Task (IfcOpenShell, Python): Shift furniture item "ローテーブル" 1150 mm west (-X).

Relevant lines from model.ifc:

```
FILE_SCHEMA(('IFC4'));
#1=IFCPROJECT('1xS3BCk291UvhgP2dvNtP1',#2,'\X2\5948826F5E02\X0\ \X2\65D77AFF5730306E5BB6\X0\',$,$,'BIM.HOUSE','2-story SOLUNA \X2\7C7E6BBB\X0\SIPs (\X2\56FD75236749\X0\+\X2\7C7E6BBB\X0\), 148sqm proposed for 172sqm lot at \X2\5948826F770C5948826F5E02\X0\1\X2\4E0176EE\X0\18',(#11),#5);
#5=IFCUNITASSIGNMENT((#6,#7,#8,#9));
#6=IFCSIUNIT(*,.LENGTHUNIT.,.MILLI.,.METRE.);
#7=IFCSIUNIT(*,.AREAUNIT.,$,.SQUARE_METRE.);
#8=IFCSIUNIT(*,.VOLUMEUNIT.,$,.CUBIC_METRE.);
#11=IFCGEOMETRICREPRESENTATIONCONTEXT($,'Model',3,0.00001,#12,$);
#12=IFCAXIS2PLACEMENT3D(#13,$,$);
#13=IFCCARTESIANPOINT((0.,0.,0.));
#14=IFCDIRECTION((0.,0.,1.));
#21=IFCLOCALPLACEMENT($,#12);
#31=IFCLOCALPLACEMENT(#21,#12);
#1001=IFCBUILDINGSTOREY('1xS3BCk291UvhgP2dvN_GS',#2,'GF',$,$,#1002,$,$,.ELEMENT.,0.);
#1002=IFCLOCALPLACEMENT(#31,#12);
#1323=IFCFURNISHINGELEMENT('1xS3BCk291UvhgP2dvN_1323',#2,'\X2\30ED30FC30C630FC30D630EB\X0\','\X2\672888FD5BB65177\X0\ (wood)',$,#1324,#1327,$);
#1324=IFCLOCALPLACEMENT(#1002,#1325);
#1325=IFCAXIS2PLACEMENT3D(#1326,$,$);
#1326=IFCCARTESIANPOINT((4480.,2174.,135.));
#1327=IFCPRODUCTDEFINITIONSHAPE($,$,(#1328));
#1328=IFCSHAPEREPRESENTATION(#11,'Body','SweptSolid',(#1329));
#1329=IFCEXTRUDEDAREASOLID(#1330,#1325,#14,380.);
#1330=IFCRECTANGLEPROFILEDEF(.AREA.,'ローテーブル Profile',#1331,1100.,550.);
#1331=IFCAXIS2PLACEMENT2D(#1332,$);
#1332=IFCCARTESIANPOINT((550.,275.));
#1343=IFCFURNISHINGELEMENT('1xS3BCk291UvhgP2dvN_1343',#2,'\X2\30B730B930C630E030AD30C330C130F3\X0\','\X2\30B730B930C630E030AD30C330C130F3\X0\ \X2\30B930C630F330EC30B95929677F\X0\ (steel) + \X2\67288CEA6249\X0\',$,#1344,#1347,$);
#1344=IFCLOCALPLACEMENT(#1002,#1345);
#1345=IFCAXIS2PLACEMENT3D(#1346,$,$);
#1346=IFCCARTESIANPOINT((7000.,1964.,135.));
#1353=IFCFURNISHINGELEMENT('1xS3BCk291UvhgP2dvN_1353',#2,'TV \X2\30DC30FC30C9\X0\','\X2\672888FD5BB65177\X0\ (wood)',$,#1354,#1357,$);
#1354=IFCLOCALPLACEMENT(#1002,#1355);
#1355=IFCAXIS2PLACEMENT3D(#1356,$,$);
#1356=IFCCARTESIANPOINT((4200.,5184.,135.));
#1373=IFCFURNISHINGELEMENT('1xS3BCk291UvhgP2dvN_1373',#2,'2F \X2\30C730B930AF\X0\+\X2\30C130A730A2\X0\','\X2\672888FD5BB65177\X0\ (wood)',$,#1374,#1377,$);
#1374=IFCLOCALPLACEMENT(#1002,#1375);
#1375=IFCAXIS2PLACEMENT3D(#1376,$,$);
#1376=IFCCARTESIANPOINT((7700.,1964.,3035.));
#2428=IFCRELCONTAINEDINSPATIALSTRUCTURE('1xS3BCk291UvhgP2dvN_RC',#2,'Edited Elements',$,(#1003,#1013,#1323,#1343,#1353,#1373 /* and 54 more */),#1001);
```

```python
import ifcopenshell
import ifcopenshell.api.geometry
import ifcopenshell.util.placement

model = ifcopenshell.open("model.ifc")

item = model.by_guid("1xS3BCk291UvhgP2dvN_1323")
matrix = ifcopenshell.util.placement.get_local_placement(item.ObjectPlacement)
matrix[0, 3] -= 1150.0
ifcopenshell.api.geometry.edit_object_placement(model, product=item, matrix=matrix, is_si=False)

print(ifcopenshell.util.placement.get_local_placement(item.ObjectPlacement).round(3) + 0.0)

model.write("model-out.ifc")
```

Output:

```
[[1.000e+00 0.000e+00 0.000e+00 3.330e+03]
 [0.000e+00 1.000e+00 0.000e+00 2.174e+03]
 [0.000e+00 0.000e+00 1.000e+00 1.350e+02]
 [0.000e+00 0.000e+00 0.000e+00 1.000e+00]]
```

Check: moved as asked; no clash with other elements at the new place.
